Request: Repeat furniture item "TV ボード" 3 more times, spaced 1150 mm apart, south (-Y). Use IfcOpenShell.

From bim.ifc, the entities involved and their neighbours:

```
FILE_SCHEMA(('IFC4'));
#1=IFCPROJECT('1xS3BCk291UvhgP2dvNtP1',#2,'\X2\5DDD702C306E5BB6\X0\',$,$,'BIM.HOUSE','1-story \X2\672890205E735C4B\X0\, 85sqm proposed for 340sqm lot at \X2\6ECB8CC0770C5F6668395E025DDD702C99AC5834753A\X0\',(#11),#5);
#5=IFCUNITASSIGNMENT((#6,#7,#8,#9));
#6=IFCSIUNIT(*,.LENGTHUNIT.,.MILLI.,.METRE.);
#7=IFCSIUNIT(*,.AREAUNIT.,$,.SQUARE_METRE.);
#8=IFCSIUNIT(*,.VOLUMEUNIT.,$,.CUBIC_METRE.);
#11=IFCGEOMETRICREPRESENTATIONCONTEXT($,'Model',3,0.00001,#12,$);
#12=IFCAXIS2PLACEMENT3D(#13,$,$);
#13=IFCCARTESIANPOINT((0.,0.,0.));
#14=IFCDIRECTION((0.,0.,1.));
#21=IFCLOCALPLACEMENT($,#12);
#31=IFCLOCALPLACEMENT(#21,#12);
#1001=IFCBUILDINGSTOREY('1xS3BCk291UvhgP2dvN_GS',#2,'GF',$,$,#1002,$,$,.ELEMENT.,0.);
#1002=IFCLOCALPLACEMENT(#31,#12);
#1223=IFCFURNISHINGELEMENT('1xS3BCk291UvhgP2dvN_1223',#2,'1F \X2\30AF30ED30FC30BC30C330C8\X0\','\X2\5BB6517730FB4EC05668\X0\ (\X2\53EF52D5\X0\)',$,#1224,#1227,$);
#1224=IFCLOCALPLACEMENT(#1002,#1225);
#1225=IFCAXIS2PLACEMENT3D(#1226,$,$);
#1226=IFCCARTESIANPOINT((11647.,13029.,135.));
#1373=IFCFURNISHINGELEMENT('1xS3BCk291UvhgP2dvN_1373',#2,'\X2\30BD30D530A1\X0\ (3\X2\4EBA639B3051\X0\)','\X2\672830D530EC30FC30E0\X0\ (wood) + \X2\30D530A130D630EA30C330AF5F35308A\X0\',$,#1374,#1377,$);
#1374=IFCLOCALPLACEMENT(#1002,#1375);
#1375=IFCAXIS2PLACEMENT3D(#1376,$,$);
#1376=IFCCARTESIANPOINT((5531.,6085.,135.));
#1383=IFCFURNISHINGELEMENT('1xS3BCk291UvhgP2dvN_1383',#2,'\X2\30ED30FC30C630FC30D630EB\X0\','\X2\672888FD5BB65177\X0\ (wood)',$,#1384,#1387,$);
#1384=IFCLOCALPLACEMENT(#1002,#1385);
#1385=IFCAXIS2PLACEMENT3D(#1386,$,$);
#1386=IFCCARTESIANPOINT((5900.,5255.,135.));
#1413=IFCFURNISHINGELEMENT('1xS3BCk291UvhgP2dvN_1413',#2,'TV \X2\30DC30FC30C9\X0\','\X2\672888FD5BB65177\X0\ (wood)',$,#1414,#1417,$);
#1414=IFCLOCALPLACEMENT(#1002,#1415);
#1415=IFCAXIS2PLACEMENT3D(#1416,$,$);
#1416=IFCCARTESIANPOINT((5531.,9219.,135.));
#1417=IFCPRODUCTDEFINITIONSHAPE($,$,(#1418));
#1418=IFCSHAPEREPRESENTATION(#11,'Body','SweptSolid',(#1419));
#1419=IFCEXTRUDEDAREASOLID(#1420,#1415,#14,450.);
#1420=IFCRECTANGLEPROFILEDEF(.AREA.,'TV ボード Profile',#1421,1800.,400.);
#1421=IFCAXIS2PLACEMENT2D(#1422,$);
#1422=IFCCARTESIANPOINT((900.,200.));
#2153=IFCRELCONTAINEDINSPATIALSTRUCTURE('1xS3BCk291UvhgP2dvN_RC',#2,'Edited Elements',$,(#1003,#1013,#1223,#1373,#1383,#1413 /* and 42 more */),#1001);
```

```python
import numpy as np
import ifcopenshell
import ifcopenshell.api.geometry
import ifcopenshell.api.root
import ifcopenshell.util.element
import ifcopenshell.util.placement

model = ifcopenshell.open("bim.ifc")


def reuse_history(source, copy):
    """copy_class also copies each property set's owner history, people and application; keep the originals."""
    for rel in copy.IsDefinedBy:
        if rel.is_a("IfcRelDefinesByProperties") and (history := rel.RelatingPropertyDefinition.OwnerHistory):
            rel.RelatingPropertyDefinition.OwnerHistory = source.OwnerHistory
            ifcopenshell.util.element.remove_deep2(model, history)


source = model.by_guid("1xS3BCk291UvhgP2dvN_1413")
base = ifcopenshell.util.placement.get_local_placement(source.ObjectPlacement)
step = np.array([0.0, -1.0, 0.0]) * 1150.0

for i in range(1, 4):
    copy = ifcopenshell.api.root.copy_class(model, product=source)
    copy.Representation = ifcopenshell.util.element.copy_deep(
        model, source.Representation, exclude=["IfcGeometricRepresentationContext", "IfcRepresentationMap"]
    )
    reuse_history(source, copy)
    matrix = base.copy()
    matrix[:3, 3] += i * step
    print("added at", matrix[:3, 3].round(3) + 0.0)
    ifcopenshell.api.geometry.edit_object_placement(model, product=copy, matrix=matrix, is_si=False)

model.write("bim_updated.ifc")
```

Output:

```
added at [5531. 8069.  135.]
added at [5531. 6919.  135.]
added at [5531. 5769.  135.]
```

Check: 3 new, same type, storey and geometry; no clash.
